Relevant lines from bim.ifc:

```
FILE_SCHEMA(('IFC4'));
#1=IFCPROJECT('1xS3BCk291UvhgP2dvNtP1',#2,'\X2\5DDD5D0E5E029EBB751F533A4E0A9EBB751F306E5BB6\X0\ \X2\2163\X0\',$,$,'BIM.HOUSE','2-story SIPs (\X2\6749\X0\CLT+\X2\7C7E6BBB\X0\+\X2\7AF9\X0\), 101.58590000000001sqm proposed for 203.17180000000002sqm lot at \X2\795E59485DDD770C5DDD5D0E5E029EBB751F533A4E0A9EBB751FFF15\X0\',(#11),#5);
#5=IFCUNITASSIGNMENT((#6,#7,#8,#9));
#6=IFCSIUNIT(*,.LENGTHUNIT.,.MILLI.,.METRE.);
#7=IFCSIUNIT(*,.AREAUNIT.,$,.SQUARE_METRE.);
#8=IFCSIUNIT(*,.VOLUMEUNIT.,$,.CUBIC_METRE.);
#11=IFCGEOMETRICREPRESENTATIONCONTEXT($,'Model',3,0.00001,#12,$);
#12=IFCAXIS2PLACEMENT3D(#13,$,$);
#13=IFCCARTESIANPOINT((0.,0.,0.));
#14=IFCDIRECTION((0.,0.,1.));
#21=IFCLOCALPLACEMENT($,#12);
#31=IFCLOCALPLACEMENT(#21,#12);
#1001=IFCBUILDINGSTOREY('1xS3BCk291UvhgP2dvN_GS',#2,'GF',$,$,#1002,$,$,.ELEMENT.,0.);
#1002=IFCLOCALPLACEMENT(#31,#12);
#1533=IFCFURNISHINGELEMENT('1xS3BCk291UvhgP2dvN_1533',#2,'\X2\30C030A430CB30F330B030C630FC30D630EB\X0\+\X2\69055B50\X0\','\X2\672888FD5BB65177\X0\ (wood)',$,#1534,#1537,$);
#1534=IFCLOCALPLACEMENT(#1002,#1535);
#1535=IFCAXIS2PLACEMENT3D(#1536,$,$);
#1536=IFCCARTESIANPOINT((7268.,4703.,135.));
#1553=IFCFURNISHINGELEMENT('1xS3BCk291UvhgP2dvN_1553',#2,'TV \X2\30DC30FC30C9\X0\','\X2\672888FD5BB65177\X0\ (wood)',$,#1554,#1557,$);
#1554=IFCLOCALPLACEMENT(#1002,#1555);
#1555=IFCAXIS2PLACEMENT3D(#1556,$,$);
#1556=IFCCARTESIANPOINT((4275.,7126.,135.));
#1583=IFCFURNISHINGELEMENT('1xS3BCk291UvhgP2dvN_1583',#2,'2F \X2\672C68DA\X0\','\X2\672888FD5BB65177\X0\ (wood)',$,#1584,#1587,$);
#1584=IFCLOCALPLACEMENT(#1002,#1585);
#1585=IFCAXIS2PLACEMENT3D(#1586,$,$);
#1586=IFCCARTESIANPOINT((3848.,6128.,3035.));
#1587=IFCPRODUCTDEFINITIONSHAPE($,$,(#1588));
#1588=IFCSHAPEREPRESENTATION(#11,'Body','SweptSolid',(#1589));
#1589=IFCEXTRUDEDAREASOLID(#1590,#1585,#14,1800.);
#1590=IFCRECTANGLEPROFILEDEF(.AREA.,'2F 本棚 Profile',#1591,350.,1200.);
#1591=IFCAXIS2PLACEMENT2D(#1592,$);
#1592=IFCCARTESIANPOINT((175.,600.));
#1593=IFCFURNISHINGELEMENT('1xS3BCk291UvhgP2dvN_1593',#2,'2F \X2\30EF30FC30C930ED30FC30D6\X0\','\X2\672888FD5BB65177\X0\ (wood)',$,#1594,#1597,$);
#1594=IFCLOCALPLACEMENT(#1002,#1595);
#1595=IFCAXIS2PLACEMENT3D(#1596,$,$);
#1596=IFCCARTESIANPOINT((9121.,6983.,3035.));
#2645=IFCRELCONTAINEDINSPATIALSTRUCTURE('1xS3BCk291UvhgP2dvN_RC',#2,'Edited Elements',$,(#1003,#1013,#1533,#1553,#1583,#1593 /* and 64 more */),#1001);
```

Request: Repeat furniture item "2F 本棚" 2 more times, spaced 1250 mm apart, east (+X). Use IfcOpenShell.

```python
import numpy as np
import ifcopenshell
import ifcopenshell.api.geometry
import ifcopenshell.api.root
import ifcopenshell.util.element
import ifcopenshell.util.placement
import ifcopenshell.util.unit

model = ifcopenshell.open("bim.ifc")
unit_scale = ifcopenshell.util.unit.calculate_unit_scale(model)


def reuse_history(source, copy):
    """copy_class also copies each property set's owner history, people and application; keep the originals."""
    for rel in copy.IsDefinedBy:
        if rel.is_a("IfcRelDefinesByProperties") and (history := rel.RelatingPropertyDefinition.OwnerHistory):
            rel.RelatingPropertyDefinition.OwnerHistory = source.OwnerHistory
            ifcopenshell.util.element.remove_deep2(model, history)


source = model.by_guid("1xS3BCk291UvhgP2dvN_1583")
base = ifcopenshell.util.placement.get_local_placement(source.ObjectPlacement)
step = np.array([1.0, 0.0, 0.0]) * 1.25 / unit_scale

for i in range(1, 3):
    copy = ifcopenshell.api.root.copy_class(model, product=source)
    copy.Representation = ifcopenshell.util.element.copy_deep(
        model, source.Representation, exclude=["IfcGeometricRepresentationContext", "IfcRepresentationMap"]
    )
    reuse_history(source, copy)
    matrix = base.copy()
    matrix[:3, 3] += i * step
    print("added at", matrix[:3, 3].round(3) + 0.0)
    ifcopenshell.api.geometry.edit_object_placement(model, product=copy, matrix=matrix, is_si=False)

model.write("bim_v2.ifc")
```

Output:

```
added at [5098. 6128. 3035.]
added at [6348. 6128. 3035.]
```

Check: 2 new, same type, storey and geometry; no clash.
